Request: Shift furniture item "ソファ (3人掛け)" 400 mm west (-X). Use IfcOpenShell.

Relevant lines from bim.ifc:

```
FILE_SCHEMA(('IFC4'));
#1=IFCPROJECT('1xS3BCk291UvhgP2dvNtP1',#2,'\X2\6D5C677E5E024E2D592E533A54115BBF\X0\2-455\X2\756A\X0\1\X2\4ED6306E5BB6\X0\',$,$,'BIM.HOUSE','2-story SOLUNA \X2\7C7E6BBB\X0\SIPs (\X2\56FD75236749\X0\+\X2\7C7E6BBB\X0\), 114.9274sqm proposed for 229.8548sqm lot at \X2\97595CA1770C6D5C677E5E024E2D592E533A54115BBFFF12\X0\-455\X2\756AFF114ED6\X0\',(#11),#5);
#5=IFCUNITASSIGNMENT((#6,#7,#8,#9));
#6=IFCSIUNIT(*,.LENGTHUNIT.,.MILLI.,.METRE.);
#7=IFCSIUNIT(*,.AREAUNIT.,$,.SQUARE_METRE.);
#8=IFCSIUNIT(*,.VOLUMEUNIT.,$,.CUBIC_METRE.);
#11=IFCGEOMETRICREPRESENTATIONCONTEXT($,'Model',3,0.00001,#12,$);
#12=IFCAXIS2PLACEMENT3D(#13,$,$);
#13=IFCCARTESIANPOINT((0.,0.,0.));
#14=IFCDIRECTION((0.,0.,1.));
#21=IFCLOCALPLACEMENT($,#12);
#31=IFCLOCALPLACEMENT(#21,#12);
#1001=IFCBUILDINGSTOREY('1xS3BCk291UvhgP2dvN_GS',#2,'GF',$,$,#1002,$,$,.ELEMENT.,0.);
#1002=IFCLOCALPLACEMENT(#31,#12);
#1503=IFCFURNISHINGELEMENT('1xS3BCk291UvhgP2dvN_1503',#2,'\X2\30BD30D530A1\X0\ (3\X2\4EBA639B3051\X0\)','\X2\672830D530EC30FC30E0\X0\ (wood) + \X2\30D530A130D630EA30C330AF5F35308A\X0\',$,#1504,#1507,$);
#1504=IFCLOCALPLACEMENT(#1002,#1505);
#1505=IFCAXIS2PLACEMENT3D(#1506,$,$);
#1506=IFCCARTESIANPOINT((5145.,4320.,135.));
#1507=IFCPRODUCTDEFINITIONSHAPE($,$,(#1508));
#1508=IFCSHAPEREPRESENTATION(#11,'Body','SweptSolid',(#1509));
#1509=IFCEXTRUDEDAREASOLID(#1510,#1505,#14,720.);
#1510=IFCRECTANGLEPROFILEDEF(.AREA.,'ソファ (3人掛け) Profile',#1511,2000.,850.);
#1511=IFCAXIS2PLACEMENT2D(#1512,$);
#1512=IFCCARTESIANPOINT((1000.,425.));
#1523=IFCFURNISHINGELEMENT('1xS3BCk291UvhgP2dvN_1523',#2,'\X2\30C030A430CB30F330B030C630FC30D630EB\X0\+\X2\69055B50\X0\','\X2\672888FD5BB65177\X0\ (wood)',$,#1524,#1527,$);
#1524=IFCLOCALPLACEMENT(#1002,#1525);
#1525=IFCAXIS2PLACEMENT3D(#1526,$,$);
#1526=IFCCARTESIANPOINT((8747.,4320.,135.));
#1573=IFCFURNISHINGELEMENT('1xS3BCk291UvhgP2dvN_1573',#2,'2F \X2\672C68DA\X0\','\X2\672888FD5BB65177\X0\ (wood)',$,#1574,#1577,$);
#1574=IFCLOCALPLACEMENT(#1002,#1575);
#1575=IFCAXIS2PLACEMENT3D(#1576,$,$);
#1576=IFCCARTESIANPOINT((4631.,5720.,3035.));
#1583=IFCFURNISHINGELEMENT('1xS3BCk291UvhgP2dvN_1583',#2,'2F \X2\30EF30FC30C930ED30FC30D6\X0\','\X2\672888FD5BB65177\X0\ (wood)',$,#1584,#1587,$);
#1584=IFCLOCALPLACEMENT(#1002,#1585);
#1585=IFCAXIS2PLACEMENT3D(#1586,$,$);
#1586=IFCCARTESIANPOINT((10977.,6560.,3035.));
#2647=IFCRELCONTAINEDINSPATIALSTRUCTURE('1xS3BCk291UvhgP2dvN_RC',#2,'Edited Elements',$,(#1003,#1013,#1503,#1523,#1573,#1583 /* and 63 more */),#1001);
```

```python
import ifcopenshell
import ifcopenshell.api.geometry
import ifcopenshell.util.placement
import ifcopenshell.util.unit

model = ifcopenshell.open("bim.ifc")
unit_scale = ifcopenshell.util.unit.calculate_unit_scale(model)

item = model.by_id(1503)
matrix = ifcopenshell.util.placement.get_local_placement(item.ObjectPlacement)
matrix[0, 3] -= 0.4 / unit_scale
ifcopenshell.api.geometry.edit_object_placement(model, product=item, matrix=matrix, is_si=False)

print(ifcopenshell.util.placement.get_local_placement(item.ObjectPlacement).round(3) + 0.0)

model.write("bim-out.ifc")
```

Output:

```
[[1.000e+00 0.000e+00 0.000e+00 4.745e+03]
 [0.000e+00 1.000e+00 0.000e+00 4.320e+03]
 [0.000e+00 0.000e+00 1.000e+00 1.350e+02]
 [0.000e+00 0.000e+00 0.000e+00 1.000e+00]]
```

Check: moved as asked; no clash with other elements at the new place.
